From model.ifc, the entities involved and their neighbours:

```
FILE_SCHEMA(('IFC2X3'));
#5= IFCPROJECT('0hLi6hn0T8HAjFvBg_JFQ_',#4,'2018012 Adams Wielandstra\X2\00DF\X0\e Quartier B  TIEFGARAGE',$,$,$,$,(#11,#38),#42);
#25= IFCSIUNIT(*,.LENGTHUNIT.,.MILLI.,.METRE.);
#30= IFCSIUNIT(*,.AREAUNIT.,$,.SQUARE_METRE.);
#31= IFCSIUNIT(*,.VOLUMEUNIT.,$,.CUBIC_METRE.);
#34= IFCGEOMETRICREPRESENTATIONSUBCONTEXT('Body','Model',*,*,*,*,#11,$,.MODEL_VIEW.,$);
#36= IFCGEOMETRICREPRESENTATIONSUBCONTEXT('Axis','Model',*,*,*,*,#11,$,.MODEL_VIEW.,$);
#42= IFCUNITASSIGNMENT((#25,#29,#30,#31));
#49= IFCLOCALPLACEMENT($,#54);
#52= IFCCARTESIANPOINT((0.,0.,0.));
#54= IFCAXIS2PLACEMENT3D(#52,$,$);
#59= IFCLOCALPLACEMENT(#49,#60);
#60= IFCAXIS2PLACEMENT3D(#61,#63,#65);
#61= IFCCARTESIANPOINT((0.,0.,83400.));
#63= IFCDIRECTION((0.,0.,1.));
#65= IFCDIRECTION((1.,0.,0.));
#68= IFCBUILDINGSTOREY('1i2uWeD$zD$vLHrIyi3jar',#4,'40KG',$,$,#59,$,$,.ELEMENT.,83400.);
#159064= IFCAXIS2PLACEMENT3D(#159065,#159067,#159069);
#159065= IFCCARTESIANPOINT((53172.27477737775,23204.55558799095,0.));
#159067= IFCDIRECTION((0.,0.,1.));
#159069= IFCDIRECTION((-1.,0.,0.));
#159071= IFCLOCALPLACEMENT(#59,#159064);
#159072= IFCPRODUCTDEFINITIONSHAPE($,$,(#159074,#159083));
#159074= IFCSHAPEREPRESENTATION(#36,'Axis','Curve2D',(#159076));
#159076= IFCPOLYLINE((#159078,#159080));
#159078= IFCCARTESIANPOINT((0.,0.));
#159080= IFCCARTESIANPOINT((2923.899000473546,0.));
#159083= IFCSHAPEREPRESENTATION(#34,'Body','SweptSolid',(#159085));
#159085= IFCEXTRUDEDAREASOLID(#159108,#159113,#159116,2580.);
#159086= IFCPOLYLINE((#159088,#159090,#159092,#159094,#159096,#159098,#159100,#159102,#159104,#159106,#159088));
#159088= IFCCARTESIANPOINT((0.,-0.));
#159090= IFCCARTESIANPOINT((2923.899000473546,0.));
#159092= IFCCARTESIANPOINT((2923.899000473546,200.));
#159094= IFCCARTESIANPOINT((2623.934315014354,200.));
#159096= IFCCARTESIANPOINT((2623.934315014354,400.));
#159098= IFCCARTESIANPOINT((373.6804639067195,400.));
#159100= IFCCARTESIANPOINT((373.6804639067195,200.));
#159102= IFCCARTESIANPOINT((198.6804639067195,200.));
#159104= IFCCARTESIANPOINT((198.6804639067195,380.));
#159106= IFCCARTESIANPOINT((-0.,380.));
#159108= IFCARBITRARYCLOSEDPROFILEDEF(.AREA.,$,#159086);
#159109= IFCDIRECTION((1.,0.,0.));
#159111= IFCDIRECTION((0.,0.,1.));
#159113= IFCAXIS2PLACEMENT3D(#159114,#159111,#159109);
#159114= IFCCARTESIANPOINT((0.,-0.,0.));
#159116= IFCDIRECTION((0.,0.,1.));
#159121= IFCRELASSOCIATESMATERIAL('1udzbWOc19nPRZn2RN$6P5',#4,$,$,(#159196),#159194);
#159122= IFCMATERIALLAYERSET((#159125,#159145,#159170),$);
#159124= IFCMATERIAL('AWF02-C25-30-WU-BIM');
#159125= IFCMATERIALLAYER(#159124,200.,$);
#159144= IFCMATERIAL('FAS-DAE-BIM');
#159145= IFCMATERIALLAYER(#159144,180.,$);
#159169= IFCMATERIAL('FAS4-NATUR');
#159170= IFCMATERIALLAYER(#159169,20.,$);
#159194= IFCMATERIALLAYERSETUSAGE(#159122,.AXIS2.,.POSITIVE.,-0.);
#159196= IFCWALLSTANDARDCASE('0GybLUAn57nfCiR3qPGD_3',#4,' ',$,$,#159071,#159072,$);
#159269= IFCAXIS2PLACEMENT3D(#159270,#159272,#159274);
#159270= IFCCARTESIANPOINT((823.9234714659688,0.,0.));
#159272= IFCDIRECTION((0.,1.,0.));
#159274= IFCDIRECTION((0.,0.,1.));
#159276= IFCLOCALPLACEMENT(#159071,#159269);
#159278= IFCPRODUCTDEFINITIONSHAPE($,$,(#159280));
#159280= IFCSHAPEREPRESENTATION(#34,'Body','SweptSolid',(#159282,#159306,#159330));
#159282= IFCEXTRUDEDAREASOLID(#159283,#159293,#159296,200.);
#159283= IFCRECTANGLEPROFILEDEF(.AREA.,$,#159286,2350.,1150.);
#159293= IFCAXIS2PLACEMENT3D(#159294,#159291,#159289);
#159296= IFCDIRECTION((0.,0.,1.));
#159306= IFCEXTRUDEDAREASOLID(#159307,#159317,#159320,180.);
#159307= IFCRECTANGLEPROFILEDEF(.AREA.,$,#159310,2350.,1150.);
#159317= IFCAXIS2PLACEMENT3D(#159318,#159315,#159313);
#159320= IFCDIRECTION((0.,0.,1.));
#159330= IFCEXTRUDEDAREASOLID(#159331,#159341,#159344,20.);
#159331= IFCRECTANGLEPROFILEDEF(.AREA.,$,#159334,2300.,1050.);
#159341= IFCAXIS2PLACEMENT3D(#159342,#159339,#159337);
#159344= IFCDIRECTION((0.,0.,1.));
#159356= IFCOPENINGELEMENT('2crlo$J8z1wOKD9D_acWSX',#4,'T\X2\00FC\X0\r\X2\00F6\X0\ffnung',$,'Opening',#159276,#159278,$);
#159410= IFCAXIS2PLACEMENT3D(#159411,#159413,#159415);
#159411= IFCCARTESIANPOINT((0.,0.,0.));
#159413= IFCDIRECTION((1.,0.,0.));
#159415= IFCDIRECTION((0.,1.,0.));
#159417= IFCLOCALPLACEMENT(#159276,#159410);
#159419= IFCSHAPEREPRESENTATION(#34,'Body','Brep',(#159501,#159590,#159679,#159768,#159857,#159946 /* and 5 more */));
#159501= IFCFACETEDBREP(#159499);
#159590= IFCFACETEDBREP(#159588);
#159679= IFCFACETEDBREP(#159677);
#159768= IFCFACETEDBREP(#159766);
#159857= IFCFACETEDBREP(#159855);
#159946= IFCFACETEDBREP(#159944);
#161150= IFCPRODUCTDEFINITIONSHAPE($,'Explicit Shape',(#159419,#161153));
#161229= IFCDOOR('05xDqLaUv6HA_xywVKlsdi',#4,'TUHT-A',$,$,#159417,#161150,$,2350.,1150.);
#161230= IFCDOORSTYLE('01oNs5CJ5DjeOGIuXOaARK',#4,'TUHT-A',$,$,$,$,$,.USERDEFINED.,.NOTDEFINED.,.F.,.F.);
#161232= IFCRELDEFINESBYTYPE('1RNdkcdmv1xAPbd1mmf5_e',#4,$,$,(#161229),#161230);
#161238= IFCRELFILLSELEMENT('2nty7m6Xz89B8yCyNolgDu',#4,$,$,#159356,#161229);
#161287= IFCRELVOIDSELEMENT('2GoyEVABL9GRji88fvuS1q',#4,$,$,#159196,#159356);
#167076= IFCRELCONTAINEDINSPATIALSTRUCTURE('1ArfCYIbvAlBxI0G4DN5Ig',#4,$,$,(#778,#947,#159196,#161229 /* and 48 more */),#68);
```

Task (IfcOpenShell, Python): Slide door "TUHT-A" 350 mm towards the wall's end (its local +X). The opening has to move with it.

```python
import ifcopenshell
import ifcopenshell.api.geometry
import ifcopenshell.util.placement
import ifcopenshell.util.unit

model = ifcopenshell.open("model.ifc")
unit_scale = ifcopenshell.util.unit.calculate_unit_scale(model)

door = model.by_id(161229)
opening = door.FillsVoids[0].RelatingOpeningElement
wall = opening.VoidsElements[0].RelatingBuildingElement

wall_matrix = ifcopenshell.util.placement.get_local_placement(wall.ObjectPlacement)
shift = wall_matrix[:3, 0] * 0.35 / unit_scale
before = ifcopenshell.util.placement.get_local_placement(door.ObjectPlacement)[:3, 3].copy()

# The door is placed relative to its opening, so it follows when the opening moves.
matrix = ifcopenshell.util.placement.get_local_placement(opening.ObjectPlacement)
matrix[:3, 3] += shift
ifcopenshell.api.geometry.edit_object_placement(
    model, product=opening, matrix=matrix, is_si=False, should_transform_children=True
)

after = ifcopenshell.util.placement.get_local_placement(door.ObjectPlacement)[:3, 3]
print("door moved by", (after - before).round(3) + 0.0)

model.write("model_rev.ifc")
```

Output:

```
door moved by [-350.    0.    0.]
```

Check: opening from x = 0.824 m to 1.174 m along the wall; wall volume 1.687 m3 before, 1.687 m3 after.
